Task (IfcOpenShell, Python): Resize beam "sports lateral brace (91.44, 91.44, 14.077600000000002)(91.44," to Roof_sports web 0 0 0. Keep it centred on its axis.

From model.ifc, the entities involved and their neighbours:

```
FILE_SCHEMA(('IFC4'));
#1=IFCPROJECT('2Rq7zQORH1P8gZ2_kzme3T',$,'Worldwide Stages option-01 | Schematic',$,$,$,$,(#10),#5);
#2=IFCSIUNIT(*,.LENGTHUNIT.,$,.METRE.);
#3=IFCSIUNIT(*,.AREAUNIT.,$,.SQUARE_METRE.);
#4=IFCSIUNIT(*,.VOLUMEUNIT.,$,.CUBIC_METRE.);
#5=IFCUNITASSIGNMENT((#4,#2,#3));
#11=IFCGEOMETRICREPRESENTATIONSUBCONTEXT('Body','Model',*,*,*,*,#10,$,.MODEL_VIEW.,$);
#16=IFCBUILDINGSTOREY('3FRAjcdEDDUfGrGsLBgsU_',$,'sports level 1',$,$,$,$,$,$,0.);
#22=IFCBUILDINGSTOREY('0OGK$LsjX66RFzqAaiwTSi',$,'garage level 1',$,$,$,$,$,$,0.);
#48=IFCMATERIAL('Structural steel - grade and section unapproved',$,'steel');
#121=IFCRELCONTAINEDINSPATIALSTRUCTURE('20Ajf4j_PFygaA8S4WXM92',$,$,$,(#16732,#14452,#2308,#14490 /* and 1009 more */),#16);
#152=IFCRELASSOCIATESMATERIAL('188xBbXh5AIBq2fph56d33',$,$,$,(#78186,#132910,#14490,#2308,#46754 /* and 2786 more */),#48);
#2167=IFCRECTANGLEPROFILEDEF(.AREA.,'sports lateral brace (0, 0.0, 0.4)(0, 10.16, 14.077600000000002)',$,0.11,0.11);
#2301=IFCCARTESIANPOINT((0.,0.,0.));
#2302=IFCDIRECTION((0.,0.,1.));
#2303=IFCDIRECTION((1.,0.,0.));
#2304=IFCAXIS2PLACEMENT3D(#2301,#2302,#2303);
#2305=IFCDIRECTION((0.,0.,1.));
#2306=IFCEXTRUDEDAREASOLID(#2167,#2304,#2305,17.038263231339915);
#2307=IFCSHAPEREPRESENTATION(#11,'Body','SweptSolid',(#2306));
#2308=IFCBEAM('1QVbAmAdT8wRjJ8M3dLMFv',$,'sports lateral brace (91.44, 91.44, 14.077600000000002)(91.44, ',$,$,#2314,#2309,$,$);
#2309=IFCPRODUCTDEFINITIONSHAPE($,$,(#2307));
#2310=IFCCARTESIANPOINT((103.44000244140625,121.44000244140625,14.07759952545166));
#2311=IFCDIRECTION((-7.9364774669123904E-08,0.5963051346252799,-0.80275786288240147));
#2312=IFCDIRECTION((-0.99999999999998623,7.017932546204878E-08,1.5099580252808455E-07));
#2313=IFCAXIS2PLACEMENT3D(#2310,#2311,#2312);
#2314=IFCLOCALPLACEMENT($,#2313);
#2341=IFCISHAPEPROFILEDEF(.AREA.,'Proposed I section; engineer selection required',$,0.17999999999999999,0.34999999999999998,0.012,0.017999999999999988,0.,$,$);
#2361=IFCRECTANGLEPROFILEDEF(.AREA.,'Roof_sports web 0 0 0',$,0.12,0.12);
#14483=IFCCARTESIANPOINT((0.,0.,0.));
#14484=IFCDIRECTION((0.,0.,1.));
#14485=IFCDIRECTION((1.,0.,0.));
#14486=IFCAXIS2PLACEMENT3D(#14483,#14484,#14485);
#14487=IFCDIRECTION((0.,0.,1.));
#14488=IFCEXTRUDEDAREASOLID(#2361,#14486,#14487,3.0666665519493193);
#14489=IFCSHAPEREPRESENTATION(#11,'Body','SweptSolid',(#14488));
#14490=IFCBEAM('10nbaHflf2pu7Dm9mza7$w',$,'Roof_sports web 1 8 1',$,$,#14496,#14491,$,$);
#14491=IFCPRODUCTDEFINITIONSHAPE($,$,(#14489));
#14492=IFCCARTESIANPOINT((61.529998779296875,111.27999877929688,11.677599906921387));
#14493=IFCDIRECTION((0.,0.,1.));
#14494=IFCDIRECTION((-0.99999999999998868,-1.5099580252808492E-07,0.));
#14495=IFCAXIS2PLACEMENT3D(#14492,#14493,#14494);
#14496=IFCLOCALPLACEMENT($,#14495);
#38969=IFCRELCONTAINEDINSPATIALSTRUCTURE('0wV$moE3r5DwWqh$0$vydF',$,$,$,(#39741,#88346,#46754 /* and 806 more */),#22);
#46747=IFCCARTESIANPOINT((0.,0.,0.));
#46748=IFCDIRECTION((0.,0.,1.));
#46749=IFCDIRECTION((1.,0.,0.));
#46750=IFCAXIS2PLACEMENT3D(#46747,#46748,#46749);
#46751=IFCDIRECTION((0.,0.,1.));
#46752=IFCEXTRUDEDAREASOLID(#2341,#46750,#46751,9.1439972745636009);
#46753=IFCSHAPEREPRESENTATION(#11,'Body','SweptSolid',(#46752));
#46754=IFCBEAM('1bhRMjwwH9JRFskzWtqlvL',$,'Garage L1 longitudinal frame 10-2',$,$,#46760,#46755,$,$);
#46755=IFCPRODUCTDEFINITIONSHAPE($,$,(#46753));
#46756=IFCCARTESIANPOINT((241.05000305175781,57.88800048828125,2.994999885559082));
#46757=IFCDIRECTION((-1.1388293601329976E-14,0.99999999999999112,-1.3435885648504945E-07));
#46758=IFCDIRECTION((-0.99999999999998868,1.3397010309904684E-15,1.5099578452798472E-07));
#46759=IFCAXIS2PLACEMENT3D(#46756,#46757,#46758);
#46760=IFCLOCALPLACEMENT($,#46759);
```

```python
import ifcopenshell
import ifcopenshell.util.element
import ifcopenshell.util.representation

model = ifcopenshell.open("model.ifc")

member = model.by_id(2308)
source = next(p for p in model.by_type("IfcRectangleProfileDef") if p.ProfileName == "Roof_sports web 0 0 0")

body = ifcopenshell.util.representation.get_representation(member, "Model", "Body")
solid = body.Items[0]
old_profile = solid.SweptArea

# Copy the section's sizes but keep this member's own profile position.
profile = ifcopenshell.util.element.copy(model, source)
profile.Position = old_profile.Position
solid.SweptArea = profile
if not model.get_total_inverses(old_profile):
    ifcopenshell.util.element.remove_deep2(model, old_profile)

print(solid.SweptArea)

model.write("model_v2.ifc")
```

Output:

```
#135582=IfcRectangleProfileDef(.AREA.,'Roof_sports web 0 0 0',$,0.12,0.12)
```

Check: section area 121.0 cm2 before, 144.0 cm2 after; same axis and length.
